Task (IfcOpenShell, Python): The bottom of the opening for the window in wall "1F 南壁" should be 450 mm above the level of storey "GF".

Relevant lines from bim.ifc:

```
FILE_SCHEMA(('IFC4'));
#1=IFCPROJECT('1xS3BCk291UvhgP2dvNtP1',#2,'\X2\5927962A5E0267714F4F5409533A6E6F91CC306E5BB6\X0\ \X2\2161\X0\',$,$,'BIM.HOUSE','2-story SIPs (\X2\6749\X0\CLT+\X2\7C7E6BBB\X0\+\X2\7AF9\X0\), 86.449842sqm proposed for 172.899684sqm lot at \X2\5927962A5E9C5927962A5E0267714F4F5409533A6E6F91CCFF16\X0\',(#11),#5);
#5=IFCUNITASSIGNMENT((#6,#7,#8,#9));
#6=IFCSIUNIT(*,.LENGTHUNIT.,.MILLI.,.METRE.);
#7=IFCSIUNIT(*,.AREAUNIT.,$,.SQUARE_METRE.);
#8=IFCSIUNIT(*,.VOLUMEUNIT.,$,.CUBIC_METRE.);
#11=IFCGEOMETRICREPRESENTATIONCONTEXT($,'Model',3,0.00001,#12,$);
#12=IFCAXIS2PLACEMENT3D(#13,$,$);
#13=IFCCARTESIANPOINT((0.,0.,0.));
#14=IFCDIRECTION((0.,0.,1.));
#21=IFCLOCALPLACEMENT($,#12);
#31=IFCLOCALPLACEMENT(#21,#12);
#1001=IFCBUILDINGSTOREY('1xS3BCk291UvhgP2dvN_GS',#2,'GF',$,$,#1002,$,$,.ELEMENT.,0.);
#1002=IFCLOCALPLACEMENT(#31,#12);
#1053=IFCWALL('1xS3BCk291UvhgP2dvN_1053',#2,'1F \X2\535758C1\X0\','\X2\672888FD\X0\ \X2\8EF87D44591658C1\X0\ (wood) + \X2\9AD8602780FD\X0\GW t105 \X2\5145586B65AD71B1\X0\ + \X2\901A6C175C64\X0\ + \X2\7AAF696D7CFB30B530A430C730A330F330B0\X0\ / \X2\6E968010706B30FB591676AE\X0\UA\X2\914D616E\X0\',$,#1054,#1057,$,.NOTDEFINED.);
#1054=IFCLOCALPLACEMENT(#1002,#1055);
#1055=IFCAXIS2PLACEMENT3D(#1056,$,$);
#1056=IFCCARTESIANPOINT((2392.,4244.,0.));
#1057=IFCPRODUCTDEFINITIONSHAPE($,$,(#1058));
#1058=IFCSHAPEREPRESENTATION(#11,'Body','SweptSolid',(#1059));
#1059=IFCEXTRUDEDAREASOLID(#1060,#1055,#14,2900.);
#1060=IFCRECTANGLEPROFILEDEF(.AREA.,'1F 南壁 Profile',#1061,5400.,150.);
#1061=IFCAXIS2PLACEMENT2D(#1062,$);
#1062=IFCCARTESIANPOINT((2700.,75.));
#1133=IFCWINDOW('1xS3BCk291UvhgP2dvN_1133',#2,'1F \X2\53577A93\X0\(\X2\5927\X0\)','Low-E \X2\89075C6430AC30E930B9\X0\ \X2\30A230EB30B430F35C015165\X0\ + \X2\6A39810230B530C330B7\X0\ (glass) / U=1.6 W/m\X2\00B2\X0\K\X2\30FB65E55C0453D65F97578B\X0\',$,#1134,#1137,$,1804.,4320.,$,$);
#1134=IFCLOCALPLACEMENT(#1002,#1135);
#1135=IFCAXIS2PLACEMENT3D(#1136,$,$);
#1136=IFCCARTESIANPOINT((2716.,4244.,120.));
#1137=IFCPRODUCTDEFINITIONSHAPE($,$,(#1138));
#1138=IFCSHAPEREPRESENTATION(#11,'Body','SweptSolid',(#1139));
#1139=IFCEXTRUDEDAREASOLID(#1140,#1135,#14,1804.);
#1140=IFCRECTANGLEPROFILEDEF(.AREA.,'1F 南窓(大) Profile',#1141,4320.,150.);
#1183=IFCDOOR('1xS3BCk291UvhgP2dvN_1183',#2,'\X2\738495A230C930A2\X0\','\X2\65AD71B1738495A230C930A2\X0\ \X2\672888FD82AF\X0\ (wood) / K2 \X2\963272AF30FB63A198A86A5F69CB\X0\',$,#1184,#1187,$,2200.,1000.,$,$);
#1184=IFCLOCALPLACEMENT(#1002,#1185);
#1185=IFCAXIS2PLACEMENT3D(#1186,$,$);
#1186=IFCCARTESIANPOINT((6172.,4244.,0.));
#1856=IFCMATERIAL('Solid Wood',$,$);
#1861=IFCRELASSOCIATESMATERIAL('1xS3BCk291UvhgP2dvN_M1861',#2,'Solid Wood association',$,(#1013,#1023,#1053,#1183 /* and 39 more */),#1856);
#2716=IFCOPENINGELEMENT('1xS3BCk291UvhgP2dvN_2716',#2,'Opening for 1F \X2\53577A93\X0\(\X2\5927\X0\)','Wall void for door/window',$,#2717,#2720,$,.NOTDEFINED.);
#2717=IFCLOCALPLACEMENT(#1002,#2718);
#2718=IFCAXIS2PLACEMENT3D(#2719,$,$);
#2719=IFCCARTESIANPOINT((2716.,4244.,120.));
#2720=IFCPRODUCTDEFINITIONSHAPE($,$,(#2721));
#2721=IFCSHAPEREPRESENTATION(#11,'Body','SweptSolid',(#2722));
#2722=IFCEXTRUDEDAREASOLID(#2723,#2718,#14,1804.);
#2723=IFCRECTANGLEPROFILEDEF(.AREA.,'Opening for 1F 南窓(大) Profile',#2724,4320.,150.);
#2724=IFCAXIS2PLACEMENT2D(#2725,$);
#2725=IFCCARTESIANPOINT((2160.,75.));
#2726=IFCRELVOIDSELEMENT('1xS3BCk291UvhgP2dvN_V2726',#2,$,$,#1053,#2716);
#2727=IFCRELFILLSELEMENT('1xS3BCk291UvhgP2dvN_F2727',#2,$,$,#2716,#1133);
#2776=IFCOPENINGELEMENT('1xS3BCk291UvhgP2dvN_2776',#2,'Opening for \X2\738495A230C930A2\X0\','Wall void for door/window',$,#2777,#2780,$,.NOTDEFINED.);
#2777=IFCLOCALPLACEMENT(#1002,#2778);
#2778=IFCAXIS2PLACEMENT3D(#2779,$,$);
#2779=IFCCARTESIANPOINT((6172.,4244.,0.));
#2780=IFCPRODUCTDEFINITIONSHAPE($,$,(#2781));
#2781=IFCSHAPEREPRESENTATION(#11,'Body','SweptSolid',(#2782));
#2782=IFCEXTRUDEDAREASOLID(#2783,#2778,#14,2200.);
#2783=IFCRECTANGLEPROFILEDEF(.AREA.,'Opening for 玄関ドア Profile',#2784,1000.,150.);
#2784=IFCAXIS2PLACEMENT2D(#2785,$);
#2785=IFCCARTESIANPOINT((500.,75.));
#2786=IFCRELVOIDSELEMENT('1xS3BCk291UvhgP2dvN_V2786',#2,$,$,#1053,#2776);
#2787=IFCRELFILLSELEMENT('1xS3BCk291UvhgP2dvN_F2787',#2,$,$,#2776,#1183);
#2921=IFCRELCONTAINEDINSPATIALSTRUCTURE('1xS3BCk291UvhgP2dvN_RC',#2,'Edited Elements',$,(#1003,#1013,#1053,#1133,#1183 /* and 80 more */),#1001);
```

```python
import numpy as np
import ifcopenshell
import ifcopenshell.api.geometry
import ifcopenshell.geom
import ifcopenshell.util.element
import ifcopenshell.util.placement
import ifcopenshell.util.shape
import ifcopenshell.util.unit

model = ifcopenshell.open("bim.ifc")
unit_scale = ifcopenshell.util.unit.calculate_unit_scale(model)

window = model.by_guid("1xS3BCk291UvhgP2dvN_1133")
opening = window.FillsVoids[0].RelatingOpeningElement
storey = ifcopenshell.util.element.get_container(window, ifc_class="IfcBuildingStorey")
level = ifcopenshell.util.placement.get_local_placement(storey.ObjectPlacement)[2, 3]

# The opening's origin need not be at the sill, so measure its lowest point.
shape = ifcopenshell.geom.create_shape(ifcopenshell.geom.settings(), opening)
bottom = ifcopenshell.util.shape.get_shape_bottom_elevation(shape, shape.geometry) / unit_scale
dz = level + 0.45 / unit_scale - bottom

shift = np.array([0.0, 0.0, dz])
# The window is not placed relative to its opening, so move both.
for product in (opening, window):
    matrix = ifcopenshell.util.placement.get_local_placement(product.ObjectPlacement)
    matrix[:3, 3] += shift
    ifcopenshell.api.geometry.edit_object_placement(model, product=product, matrix=matrix, is_si=False)

print(f"moved by {dz * unit_scale:+.3f} m")

model.write("bim-out.ifc")
```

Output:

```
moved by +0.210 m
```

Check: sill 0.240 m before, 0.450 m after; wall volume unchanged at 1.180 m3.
